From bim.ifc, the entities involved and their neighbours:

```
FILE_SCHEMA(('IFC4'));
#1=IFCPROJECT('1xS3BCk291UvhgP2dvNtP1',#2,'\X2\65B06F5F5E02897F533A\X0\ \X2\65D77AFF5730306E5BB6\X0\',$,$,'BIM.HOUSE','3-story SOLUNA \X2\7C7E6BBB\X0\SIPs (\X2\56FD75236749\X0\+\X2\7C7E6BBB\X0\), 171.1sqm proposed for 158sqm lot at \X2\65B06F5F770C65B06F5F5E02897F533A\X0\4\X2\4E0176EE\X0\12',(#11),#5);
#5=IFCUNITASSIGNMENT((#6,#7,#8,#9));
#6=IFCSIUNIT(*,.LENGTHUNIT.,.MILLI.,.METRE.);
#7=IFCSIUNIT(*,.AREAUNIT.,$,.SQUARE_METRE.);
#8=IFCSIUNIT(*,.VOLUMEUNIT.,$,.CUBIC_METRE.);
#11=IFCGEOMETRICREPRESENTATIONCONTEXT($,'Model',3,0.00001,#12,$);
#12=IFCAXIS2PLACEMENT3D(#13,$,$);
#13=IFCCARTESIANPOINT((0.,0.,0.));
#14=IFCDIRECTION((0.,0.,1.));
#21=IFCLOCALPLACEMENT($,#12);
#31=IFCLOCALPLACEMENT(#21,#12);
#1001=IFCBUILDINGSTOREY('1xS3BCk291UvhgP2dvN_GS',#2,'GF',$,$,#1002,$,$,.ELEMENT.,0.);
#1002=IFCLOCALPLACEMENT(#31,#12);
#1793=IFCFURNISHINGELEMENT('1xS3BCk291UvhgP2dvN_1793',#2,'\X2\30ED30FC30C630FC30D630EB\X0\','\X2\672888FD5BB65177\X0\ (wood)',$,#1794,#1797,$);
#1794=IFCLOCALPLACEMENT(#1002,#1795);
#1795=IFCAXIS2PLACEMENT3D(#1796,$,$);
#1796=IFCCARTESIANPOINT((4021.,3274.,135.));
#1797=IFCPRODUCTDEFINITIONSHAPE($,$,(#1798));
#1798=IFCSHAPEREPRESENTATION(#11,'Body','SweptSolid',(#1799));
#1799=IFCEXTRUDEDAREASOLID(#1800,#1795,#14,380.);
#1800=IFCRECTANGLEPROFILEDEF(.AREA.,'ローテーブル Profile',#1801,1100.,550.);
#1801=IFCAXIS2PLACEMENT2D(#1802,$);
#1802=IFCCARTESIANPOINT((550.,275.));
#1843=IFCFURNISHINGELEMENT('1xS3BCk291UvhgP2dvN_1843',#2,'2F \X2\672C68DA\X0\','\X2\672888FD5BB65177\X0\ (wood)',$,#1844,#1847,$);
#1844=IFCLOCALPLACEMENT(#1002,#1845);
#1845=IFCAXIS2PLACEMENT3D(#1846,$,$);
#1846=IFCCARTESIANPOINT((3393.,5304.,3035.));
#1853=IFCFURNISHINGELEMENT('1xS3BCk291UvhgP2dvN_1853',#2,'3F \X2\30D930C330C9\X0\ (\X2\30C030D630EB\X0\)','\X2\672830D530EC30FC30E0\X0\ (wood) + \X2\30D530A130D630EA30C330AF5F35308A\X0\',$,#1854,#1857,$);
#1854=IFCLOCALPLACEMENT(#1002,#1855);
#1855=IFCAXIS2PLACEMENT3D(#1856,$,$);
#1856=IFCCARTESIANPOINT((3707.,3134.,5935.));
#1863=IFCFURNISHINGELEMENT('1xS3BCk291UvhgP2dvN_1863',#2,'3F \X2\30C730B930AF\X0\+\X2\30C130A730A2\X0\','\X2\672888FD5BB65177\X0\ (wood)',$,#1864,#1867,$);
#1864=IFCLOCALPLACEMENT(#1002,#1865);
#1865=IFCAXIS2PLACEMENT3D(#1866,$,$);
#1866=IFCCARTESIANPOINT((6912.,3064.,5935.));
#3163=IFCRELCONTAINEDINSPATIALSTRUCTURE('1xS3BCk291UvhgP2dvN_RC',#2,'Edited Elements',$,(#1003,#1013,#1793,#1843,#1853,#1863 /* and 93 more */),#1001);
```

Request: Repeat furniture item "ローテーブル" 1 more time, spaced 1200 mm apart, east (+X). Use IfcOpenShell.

```python
import numpy as np
import ifcopenshell
import ifcopenshell.api.geometry
import ifcopenshell.api.root
import ifcopenshell.util.element
import ifcopenshell.util.placement
import ifcopenshell.util.unit

model = ifcopenshell.open("bim.ifc")
unit_scale = ifcopenshell.util.unit.calculate_unit_scale(model)


def reuse_history(source, copy):
    """copy_class also copies each property set's owner history, people and application; keep the originals."""
    for rel in copy.IsDefinedBy:
        if rel.is_a("IfcRelDefinesByProperties") and (history := rel.RelatingPropertyDefinition.OwnerHistory):
            rel.RelatingPropertyDefinition.OwnerHistory = source.OwnerHistory
            ifcopenshell.util.element.remove_deep2(model, history)


source = model.by_id(1793)
base = ifcopenshell.util.placement.get_local_placement(source.ObjectPlacement)
step = np.array([1.0, 0.0, 0.0]) * 1.2 / unit_scale

for i in range(1, 2):
    copy = ifcopenshell.api.root.copy_class(model, product=source)
    copy.Representation = ifcopenshell.util.element.copy_deep(
        model, source.Representation, exclude=["IfcGeometricRepresentationContext", "IfcRepresentationMap"]
    )
    reuse_history(source, copy)
    matrix = base.copy()
    matrix[:3, 3] += i * step
    print("added at", matrix[:3, 3].round(3) + 0.0)
    ifcopenshell.api.geometry.edit_object_placement(model, product=copy, matrix=matrix, is_si=False)

model.write("bim_rev.ifc")
```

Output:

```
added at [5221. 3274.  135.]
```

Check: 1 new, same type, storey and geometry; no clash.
